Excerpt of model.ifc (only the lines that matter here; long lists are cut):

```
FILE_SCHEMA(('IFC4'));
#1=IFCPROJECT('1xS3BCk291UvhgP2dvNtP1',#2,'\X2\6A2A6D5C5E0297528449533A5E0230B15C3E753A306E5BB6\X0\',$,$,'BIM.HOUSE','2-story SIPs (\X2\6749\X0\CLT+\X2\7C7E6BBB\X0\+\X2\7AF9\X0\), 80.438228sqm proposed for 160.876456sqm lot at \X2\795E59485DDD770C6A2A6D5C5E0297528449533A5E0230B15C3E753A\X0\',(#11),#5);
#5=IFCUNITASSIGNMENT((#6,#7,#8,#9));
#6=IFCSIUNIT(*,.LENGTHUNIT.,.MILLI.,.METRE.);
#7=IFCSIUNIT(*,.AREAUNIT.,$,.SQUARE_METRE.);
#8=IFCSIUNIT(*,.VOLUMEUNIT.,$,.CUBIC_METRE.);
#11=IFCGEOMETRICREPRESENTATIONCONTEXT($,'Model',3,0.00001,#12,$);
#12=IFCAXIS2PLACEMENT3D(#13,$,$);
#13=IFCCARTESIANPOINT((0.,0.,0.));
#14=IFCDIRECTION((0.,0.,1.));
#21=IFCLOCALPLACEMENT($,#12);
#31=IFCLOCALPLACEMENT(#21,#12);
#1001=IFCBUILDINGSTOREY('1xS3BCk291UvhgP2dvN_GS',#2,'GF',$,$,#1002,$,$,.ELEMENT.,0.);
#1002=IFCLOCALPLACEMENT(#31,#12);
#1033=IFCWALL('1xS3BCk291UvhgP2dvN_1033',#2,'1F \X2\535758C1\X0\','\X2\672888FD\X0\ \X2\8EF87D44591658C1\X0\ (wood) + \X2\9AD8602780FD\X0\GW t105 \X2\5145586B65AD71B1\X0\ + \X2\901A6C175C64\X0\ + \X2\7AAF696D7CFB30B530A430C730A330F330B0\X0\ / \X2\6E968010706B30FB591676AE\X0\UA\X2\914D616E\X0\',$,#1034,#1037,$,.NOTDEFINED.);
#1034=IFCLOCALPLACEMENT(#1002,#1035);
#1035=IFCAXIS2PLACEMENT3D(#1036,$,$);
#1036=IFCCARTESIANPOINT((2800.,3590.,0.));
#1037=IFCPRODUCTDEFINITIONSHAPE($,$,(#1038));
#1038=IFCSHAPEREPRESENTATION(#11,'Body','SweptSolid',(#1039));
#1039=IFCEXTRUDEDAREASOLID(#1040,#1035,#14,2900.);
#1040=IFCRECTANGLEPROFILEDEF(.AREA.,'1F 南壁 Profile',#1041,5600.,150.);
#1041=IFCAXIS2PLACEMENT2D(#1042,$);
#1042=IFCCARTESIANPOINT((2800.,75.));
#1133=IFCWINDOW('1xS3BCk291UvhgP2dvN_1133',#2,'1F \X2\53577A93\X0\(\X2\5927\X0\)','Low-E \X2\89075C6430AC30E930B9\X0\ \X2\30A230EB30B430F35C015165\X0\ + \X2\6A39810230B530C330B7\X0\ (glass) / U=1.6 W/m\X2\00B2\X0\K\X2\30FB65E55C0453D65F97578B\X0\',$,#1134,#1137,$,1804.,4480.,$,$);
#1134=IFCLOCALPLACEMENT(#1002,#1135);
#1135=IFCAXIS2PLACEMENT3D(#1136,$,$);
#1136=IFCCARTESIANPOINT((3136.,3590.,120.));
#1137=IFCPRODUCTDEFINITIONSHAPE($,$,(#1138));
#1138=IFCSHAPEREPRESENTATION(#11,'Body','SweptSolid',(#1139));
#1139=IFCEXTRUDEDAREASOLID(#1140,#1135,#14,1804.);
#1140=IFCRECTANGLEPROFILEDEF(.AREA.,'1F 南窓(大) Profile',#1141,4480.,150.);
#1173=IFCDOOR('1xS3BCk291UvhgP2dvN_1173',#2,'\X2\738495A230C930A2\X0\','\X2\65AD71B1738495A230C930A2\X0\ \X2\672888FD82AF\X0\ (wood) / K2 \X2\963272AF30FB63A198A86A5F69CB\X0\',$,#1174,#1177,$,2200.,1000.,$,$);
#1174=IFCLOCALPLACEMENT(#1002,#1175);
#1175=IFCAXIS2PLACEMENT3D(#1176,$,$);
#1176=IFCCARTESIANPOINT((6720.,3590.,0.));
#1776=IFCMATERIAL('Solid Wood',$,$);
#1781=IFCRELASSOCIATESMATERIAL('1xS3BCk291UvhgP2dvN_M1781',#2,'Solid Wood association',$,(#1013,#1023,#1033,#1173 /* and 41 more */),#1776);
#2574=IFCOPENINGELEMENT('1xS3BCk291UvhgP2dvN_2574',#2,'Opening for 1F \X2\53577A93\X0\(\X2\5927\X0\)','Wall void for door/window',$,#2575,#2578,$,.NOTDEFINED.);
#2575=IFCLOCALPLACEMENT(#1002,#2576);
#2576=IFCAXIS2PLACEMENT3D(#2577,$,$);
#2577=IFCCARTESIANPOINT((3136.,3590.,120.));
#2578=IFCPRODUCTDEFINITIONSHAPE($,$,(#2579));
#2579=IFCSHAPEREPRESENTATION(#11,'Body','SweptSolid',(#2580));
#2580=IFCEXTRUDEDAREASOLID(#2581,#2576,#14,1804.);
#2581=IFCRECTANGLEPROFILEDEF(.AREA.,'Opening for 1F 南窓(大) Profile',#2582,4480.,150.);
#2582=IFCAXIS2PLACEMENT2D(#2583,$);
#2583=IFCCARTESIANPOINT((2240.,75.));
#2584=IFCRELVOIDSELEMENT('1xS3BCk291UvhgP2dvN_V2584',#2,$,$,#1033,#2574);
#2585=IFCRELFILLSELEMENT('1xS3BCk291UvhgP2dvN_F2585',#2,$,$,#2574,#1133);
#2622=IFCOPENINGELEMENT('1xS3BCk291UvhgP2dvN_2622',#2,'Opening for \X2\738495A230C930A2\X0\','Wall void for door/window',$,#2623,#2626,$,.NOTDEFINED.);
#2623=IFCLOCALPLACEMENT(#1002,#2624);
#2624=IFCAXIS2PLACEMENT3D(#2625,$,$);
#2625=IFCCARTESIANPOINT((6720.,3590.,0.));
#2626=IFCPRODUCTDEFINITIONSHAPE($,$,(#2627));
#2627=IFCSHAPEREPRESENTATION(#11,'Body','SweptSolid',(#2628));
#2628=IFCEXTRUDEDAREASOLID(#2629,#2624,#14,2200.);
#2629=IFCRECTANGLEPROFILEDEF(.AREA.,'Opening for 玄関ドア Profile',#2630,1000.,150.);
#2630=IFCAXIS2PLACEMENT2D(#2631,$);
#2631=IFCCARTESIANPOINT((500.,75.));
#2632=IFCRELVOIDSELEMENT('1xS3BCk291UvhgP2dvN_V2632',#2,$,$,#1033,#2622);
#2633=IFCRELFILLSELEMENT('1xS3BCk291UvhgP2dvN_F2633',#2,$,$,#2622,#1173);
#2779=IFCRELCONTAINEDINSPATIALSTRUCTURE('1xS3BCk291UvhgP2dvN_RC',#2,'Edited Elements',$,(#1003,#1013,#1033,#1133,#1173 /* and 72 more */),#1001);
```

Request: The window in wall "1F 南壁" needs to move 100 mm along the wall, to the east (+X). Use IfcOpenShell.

```python
import ifcopenshell
import ifcopenshell.api.geometry
import ifcopenshell.util.placement

model = ifcopenshell.open("model.ifc")

window = model.by_guid("1xS3BCk291UvhgP2dvN_1133")
opening = window.FillsVoids[0].RelatingOpeningElement
wall = opening.VoidsElements[0].RelatingBuildingElement

wall_matrix = ifcopenshell.util.placement.get_local_placement(wall.ObjectPlacement)
shift = wall_matrix[:3, 0] * 100.0
before = ifcopenshell.util.placement.get_local_placement(window.ObjectPlacement)[:3, 3].copy()

# The window is not placed relative to its opening, so move both.
for product in (opening, window):
    matrix = ifcopenshell.util.placement.get_local_placement(product.ObjectPlacement)
    matrix[:3, 3] += shift
    ifcopenshell.api.geometry.edit_object_placement(model, product=product, matrix=matrix, is_si=False)

after = ifcopenshell.util.placement.get_local_placement(window.ObjectPlacement)[:3, 3]
print("window moved by", (after - before).round(3) + 0.0)

model.write("model-out.ifc")
```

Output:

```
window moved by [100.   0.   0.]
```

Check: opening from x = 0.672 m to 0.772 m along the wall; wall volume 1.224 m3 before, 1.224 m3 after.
